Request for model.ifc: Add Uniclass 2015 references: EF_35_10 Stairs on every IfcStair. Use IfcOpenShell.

First a look at what the model holds.

```python
import ifcopenshell

model = ifcopenshell.open("model.ifc")
print(model.schema)
print("classifications:", [c.Name for c in model.by_type("IfcClassification")])
for ifc_class in ("IfcDoor", "IfcRoof", "IfcStair", "IfcWall", "IfcWindow"):
    print(ifc_class, len(model.by_type(ifc_class)))
```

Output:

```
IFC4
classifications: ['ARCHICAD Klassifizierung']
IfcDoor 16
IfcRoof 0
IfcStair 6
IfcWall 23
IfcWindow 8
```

```python
import ifcopenshell
import ifcopenshell.api.classification

model = ifcopenshell.open("model.ifc")

system = ifcopenshell.api.classification.add_classification(model, classification="Uniclass 2015")

codes = {
    "IfcStair": ("EF_35_10", "Stairs"),
}
for ifc_class, (code, name) in codes.items():
    products = model.by_type(ifc_class)
    ifcopenshell.api.classification.add_reference(
        model, products=products, classification=system, identification=code, name=name
    )
    print(code, len(products))

model.write("model-out.ifc")
```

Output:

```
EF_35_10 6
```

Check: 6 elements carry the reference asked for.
